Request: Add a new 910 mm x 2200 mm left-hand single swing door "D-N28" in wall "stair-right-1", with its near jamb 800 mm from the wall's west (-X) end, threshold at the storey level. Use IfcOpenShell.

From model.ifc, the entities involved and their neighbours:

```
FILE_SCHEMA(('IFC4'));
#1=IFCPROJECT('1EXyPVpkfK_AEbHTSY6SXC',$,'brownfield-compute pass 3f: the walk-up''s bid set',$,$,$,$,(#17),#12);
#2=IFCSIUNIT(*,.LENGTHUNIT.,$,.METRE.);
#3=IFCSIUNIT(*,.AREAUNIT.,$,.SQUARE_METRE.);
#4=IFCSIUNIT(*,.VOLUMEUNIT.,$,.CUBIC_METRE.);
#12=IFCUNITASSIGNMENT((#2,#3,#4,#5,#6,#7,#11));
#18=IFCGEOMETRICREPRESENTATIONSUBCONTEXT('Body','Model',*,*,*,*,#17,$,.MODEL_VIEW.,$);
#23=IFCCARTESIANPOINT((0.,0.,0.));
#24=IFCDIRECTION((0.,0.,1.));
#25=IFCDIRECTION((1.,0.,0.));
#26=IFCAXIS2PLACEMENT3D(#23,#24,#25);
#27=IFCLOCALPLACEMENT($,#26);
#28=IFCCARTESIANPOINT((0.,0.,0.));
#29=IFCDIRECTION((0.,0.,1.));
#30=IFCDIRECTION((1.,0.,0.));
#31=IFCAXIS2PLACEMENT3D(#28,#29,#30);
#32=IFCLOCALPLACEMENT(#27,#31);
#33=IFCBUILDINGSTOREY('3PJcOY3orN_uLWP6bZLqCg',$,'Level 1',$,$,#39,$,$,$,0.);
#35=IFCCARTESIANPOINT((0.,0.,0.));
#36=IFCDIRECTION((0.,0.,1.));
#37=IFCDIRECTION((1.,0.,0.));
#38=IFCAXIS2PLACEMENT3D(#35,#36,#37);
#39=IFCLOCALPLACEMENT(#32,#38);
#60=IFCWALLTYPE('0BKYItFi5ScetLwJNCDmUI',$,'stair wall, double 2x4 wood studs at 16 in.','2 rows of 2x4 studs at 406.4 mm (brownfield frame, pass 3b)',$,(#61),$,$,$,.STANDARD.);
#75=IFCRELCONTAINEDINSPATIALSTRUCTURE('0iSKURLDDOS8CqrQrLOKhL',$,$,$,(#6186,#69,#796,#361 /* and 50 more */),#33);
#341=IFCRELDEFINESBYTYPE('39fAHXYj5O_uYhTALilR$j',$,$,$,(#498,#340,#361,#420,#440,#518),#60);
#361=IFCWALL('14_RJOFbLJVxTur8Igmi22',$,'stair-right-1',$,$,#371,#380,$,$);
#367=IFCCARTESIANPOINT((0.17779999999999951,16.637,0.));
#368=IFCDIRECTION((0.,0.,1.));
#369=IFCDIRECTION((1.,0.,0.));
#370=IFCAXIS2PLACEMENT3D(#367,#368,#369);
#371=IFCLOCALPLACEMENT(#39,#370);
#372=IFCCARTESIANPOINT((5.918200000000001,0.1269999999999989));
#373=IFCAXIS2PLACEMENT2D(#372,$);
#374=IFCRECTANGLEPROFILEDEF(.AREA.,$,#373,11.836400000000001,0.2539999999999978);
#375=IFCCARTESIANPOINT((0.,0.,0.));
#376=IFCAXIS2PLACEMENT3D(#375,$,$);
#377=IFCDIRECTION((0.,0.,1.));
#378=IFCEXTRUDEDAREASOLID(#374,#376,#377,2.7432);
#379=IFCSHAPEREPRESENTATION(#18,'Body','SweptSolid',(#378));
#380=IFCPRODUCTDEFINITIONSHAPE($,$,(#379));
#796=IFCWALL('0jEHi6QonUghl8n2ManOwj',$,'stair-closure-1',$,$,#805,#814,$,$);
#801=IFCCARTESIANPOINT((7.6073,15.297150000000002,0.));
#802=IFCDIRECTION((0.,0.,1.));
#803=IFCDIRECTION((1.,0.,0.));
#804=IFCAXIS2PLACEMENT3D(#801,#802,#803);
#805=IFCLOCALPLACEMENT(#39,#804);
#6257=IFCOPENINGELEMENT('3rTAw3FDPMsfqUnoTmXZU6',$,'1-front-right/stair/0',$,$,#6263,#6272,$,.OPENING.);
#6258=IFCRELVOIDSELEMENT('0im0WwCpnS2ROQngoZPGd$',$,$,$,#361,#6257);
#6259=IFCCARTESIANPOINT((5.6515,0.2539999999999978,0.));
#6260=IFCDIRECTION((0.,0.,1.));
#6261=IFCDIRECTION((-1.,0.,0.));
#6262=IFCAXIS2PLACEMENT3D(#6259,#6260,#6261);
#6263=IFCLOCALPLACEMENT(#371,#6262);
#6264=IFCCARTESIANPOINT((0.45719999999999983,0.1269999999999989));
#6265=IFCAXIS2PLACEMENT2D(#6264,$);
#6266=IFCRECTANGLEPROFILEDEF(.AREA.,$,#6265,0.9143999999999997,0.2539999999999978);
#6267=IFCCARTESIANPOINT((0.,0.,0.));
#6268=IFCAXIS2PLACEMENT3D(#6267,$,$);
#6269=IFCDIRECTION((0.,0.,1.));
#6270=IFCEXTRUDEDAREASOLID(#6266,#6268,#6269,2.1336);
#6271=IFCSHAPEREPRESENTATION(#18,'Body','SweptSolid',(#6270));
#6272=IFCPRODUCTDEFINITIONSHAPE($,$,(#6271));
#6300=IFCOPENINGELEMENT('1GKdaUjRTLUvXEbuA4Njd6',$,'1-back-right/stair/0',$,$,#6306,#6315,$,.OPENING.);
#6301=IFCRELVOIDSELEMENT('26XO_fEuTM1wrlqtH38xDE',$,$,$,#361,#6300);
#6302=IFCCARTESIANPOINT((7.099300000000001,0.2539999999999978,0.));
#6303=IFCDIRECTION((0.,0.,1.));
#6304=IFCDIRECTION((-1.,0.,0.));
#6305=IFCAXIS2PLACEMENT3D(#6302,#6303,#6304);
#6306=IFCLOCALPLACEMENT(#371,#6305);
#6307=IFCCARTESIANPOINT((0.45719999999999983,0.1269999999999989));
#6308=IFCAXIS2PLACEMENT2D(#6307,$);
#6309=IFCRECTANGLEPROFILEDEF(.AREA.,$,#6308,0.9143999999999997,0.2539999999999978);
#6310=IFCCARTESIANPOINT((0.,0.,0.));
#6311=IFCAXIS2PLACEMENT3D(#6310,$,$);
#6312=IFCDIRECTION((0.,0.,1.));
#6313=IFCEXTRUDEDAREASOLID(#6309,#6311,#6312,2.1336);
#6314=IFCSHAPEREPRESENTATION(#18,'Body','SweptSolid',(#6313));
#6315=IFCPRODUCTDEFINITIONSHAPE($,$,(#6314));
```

```python
import numpy as np
import ifcopenshell
import ifcopenshell.api.feature
import ifcopenshell.api.geometry
import ifcopenshell.api.root
import ifcopenshell.api.spatial
import ifcopenshell.geom
import ifcopenshell.util.element
import ifcopenshell.util.placement
import ifcopenshell.util.representation
import ifcopenshell.util.shape
import ifcopenshell.util.unit

model = ifcopenshell.open("model.ifc")
unit_scale = ifcopenshell.util.unit.calculate_unit_scale(model)
settings = ifcopenshell.geom.settings()


def volume(element):
    """Net volume in cubic metres, openings subtracted."""
    shape = ifcopenshell.geom.create_shape(settings, element)
    return ifcopenshell.util.shape.get_volume(shape.geometry)


wall = model.by_id(361)
storey = ifcopenshell.util.element.get_container(wall, ifc_class="IfcBuildingStorey")
context = ifcopenshell.util.representation.get_context(model, "Model", "Body", "MODEL_VIEW")
before = volume(wall)

width, height, from_end, sill = 0.91, 2.2, 0.8, 0.0  # metres

# The wall runs along its own X axis, and the end named is its -X end.
wall_shape = ifcopenshell.geom.create_shape(settings, wall)
x, y, z = ifcopenshell.util.shape.get_vertices(wall_shape.geometry).T
start = x.min() + from_end
face, thickness = float(y.min()), float(y.max() - y.min())
wall_matrix = ifcopenshell.util.placement.get_local_placement(wall.ObjectPlacement)
level = ifcopenshell.util.placement.get_local_placement(storey.ObjectPlacement)[2, 3]


def in_wall(x, y):
    """Placement at x, y metres in the wall's axes, at sill height."""
    matrix = wall_matrix.copy()
    matrix[:, 3] = wall_matrix @ np.array([x / unit_scale, y / unit_scale, 0.0, 1.0])
    matrix[2, 3] = level + sill / unit_scale
    return matrix


# Opening: a box that overshoots both wall faces by 50 mm.
opening = ifcopenshell.api.root.create_entity(model, ifc_class="IfcOpeningElement", predefined_type="OPENING")
box = ifcopenshell.api.geometry.add_wall_representation(
    model, context=context, length=width, height=height, thickness=thickness + 0.1
)
ifcopenshell.api.geometry.assign_representation(model, product=opening, representation=box)
ifcopenshell.api.geometry.edit_object_placement(model, product=opening, matrix=in_wall(start, face - 0.05), is_si=False)
ifcopenshell.api.feature.add_feature(model, feature=opening, element=wall)

door = ifcopenshell.api.root.create_entity(model, ifc_class="IfcDoor", name="D-N28", predefined_type="DOOR")
door.OverallWidth, door.OverallHeight = width / unit_scale, height / unit_scale
door.OperationType = "SINGLE_SWING_LEFT"
body = ifcopenshell.api.geometry.add_door_representation(
    model,
    context=context,
    overall_width=door.OverallWidth,
    overall_height=door.OverallHeight,
    operation_type="SINGLE_SWING_LEFT",
    lining_properties={"LiningDepth": thickness / unit_scale, "ThresholdDepth": thickness / unit_scale},
)
ifcopenshell.api.geometry.assign_representation(model, product=door, representation=body)
ifcopenshell.api.spatial.assign_container(model, products=[door], relating_structure=storey)
ifcopenshell.api.feature.add_filling(model, opening=opening, element=door)

# The lining spans the wall, so the door starts at the wall face.
ifcopenshell.api.geometry.edit_object_placement(model, product=door, matrix=in_wall(start, face), is_si=False)

after = volume(wall)

print(f"wall volume {before:.3f} -> {after:.3f} m3")

model.write("model-out.ifc")
```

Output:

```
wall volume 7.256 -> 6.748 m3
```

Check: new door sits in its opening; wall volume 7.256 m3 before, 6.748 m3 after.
